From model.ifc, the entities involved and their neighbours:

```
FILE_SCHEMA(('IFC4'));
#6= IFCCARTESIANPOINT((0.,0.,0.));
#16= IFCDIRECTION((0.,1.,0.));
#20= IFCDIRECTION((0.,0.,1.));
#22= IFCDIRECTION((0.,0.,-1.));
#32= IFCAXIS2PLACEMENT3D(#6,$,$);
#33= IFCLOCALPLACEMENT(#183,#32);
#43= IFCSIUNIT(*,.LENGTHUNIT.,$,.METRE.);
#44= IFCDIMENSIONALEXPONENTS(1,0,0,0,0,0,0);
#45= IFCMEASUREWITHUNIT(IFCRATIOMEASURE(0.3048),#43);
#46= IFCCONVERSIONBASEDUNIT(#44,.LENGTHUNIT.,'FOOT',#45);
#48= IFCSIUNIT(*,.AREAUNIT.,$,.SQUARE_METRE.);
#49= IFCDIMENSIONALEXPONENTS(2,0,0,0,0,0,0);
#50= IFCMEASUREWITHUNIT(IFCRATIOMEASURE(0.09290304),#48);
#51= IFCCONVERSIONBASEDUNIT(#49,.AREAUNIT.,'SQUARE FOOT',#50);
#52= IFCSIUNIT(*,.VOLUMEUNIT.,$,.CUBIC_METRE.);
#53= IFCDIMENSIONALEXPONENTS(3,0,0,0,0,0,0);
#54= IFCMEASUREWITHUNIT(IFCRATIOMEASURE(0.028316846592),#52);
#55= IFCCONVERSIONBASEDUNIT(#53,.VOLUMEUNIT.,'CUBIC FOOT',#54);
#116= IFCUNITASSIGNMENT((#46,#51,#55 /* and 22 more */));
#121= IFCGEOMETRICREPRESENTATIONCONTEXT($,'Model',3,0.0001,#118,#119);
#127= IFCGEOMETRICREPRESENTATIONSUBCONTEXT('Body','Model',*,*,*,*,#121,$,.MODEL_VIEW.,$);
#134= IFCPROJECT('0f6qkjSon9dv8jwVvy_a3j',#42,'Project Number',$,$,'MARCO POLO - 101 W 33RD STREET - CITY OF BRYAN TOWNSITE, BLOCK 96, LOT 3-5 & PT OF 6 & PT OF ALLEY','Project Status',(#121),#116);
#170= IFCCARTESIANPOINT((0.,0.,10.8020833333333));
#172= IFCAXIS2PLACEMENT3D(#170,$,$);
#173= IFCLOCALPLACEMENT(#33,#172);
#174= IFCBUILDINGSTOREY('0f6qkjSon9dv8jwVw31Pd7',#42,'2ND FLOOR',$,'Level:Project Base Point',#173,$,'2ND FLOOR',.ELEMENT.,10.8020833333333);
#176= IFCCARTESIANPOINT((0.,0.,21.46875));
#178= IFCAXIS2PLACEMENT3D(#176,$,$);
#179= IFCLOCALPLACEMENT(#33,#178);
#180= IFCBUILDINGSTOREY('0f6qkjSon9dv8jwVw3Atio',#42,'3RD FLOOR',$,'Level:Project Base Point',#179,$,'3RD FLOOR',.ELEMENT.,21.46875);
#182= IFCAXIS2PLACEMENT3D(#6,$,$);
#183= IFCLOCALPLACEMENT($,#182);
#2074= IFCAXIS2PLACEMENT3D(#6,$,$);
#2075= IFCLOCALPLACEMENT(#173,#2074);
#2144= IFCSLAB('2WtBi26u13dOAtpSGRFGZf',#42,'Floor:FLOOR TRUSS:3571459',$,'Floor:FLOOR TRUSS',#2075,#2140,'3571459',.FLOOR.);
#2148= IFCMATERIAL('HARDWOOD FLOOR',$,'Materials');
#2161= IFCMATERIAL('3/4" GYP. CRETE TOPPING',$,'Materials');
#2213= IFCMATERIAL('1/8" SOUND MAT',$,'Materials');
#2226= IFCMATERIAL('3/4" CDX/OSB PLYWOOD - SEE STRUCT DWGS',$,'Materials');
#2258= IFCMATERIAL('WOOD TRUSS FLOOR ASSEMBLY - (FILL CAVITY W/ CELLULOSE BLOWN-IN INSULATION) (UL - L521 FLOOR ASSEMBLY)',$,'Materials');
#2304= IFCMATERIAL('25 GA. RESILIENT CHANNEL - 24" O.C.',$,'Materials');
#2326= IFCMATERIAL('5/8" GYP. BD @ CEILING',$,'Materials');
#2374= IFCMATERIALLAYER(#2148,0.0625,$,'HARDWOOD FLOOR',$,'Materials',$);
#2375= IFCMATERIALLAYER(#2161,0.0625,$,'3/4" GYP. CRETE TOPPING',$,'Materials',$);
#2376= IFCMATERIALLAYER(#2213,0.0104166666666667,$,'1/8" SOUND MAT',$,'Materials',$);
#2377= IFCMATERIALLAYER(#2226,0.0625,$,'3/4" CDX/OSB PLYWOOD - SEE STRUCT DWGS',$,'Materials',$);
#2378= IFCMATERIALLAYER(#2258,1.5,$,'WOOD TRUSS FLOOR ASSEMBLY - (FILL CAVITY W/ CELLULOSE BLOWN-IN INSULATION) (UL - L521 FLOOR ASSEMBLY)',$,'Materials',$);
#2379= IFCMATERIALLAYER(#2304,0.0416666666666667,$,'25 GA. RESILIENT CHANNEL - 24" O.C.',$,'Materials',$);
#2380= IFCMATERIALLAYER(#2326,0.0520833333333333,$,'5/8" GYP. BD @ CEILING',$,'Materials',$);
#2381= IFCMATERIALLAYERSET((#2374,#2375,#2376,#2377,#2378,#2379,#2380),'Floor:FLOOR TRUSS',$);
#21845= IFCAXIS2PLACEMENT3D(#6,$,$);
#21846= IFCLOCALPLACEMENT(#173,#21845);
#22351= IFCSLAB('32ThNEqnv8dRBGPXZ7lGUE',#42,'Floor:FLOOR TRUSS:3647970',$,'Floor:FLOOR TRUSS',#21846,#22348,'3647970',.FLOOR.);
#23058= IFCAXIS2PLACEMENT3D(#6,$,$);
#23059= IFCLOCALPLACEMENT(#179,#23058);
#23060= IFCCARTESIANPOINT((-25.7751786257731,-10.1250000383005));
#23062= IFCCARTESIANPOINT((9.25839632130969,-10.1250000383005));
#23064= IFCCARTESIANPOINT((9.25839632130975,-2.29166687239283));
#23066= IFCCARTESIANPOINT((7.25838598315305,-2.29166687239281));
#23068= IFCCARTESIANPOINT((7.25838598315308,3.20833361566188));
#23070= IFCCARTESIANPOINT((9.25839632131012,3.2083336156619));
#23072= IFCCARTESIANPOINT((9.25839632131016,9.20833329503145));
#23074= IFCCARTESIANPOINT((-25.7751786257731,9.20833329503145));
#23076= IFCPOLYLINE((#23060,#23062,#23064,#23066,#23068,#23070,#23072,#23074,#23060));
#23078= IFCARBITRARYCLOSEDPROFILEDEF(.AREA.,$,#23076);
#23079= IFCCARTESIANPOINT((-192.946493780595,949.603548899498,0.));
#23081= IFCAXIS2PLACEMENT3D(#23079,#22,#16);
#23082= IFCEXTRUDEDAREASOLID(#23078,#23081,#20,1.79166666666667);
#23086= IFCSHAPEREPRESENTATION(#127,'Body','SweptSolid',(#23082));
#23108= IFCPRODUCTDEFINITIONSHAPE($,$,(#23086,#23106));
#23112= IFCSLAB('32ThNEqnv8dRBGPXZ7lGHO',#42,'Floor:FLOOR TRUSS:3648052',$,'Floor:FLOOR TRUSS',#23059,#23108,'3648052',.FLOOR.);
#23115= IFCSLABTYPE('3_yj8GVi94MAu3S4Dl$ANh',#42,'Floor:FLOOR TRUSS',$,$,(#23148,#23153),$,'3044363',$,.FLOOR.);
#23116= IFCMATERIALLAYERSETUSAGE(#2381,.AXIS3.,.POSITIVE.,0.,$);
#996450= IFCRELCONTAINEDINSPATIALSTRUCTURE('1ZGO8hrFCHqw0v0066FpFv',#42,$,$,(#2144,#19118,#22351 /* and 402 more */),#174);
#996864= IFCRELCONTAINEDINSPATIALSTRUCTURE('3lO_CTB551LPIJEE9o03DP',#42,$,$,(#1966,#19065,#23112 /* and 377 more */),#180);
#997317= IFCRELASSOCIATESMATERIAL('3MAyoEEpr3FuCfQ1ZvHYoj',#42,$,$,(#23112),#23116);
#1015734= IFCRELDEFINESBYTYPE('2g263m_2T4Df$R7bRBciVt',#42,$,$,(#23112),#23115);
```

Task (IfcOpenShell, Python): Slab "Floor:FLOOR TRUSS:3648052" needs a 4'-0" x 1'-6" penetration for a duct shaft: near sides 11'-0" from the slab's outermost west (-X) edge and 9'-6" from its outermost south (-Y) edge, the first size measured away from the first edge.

```python
import numpy as np
import ifcopenshell
import ifcopenshell.api.feature
import ifcopenshell.api.geometry
import ifcopenshell.api.root
import ifcopenshell.geom
import ifcopenshell.util.placement
import ifcopenshell.util.representation
import ifcopenshell.util.shape
import ifcopenshell.util.unit

model = ifcopenshell.open("model.ifc")
unit_scale = ifcopenshell.util.unit.calculate_unit_scale(model)
settings = ifcopenshell.geom.settings()


def volume(element):
    """Net volume in cubic metres, openings subtracted."""
    shape = ifcopenshell.geom.create_shape(settings, element)
    return ifcopenshell.util.shape.get_volume(shape.geometry)


slab = model.by_guid("32ThNEqnv8dRBGPXZ7lGHO")
before = volume(slab)

# Extent in the slab's own axes, in metres. The edges named are its -X and -Y sides.
slab_shape = ifcopenshell.geom.create_shape(settings, slab)
vertices = ifcopenshell.util.shape.get_vertices(slab_shape.geometry)
x_min, y_min, bottom = vertices.min(axis=0)
top = vertices[:, 2].max()

opening = ifcopenshell.api.root.create_entity(model, ifc_class="IfcOpeningElement", name="Duct shaft opening", predefined_type="OPENING")
context = ifcopenshell.util.representation.get_context(model, "Model", "Body", "MODEL_VIEW")
width, depth = 1.2192, 0.4572
outline = [(0.0, 0.0), (width, 0.0), (width, depth), (0.0, depth), (0.0, 0.0)]
# Overshoot both faces by 50 mm so the cut is clean.
shape = ifcopenshell.api.geometry.add_slab_representation(
    model, context=context, depth=top - bottom + 0.1, polyline=outline
)
ifcopenshell.api.geometry.assign_representation(model, product=opening, representation=shape)

matrix = ifcopenshell.util.placement.get_local_placement(slab.ObjectPlacement)
matrix[:, 3] = matrix @ np.append(np.array([x_min + 3.3528, y_min + 2.8956, bottom - 0.05]) / unit_scale, 1.0)
ifcopenshell.api.geometry.edit_object_placement(model, product=opening, matrix=matrix, is_si=False)
ifcopenshell.api.feature.add_feature(model, feature=opening, element=slab)

after = volume(slab)

print(f"slab volume {before:.3f} -> {after:.3f} m3")

model.write("model-out.ifc")
```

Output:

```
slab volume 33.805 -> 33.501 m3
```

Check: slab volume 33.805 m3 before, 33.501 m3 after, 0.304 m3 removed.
